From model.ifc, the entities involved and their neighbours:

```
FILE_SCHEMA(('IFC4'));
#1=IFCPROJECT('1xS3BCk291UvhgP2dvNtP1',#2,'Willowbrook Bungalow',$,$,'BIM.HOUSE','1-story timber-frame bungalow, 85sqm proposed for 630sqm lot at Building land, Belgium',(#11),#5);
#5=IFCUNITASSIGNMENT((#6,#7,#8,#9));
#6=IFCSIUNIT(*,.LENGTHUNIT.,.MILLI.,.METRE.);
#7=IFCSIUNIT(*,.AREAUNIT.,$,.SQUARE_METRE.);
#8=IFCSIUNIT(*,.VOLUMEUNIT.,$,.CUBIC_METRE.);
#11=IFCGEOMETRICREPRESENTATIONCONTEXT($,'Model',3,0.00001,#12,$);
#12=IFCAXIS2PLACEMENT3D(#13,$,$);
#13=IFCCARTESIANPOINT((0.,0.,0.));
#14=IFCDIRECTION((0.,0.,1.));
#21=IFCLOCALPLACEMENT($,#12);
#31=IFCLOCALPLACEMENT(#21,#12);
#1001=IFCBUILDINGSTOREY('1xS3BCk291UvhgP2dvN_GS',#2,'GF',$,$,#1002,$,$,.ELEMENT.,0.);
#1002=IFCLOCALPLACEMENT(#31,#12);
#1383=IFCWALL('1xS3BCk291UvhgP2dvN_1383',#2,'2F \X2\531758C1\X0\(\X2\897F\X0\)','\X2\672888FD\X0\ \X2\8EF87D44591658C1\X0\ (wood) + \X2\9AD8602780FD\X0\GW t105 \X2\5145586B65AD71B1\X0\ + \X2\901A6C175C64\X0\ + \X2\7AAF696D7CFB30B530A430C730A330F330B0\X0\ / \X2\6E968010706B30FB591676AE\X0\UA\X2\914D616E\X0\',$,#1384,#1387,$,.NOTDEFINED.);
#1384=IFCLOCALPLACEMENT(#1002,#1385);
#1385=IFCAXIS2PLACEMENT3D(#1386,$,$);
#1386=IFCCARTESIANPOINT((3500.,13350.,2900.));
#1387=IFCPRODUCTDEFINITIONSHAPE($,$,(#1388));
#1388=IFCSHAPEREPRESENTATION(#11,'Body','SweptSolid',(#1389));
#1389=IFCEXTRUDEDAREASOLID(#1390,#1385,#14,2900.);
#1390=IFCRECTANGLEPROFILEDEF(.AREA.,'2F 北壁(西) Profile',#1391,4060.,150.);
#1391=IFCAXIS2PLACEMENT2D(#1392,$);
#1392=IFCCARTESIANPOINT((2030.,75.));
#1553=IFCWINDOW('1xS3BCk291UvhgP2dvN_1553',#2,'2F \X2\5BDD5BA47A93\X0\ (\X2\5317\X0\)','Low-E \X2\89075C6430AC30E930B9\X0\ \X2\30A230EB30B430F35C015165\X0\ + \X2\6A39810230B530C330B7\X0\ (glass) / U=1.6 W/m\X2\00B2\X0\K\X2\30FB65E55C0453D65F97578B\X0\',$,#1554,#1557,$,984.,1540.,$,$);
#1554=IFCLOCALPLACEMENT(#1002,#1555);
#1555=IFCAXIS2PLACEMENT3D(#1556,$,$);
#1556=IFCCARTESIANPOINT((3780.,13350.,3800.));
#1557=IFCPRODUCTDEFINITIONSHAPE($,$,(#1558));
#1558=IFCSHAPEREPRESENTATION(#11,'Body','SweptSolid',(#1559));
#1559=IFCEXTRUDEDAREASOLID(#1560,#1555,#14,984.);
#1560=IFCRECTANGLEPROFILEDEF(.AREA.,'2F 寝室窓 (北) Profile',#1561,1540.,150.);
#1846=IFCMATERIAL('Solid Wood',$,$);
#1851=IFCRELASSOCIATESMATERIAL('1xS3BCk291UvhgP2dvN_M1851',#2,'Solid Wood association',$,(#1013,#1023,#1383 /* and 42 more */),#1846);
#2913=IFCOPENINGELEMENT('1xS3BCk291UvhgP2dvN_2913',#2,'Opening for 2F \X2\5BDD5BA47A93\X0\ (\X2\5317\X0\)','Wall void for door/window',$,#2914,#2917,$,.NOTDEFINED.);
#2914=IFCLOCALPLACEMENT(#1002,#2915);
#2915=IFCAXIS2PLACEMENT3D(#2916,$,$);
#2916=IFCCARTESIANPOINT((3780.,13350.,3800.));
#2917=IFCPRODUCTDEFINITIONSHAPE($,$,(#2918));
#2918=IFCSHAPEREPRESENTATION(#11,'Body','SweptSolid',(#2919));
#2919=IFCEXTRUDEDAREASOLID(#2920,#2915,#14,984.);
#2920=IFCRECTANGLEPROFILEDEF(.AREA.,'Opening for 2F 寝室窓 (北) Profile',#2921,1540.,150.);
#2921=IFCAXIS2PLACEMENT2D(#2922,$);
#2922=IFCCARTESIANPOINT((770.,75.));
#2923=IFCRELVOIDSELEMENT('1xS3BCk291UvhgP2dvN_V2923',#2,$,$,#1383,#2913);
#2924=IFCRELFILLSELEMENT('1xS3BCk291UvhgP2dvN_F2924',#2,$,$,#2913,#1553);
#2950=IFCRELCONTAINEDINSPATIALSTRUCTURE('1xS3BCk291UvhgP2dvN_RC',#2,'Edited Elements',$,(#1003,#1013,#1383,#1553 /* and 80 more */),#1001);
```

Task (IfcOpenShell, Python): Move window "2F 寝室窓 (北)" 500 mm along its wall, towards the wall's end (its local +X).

```python
import ifcopenshell
import ifcopenshell.api.geometry
import ifcopenshell.util.placement

model = ifcopenshell.open("model.ifc")

window = model.by_guid("1xS3BCk291UvhgP2dvN_1553")
opening = window.FillsVoids[0].RelatingOpeningElement
wall = opening.VoidsElements[0].RelatingBuildingElement

wall_matrix = ifcopenshell.util.placement.get_local_placement(wall.ObjectPlacement)
shift = wall_matrix[:3, 0] * 500.0
before = ifcopenshell.util.placement.get_local_placement(window.ObjectPlacement)[:3, 3].copy()

# The window is not placed relative to its opening, so move both.
for product in (opening, window):
    matrix = ifcopenshell.util.placement.get_local_placement(product.ObjectPlacement)
    matrix[:3, 3] += shift
    ifcopenshell.api.geometry.edit_object_placement(model, product=product, matrix=matrix, is_si=False)

after = ifcopenshell.util.placement.get_local_placement(window.ObjectPlacement)[:3, 3]
print("window moved by", (after - before).round(3) + 0.0)

model.write("model_edited.ifc")
```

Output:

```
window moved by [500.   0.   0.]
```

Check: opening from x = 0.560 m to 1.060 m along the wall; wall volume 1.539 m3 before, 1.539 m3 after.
